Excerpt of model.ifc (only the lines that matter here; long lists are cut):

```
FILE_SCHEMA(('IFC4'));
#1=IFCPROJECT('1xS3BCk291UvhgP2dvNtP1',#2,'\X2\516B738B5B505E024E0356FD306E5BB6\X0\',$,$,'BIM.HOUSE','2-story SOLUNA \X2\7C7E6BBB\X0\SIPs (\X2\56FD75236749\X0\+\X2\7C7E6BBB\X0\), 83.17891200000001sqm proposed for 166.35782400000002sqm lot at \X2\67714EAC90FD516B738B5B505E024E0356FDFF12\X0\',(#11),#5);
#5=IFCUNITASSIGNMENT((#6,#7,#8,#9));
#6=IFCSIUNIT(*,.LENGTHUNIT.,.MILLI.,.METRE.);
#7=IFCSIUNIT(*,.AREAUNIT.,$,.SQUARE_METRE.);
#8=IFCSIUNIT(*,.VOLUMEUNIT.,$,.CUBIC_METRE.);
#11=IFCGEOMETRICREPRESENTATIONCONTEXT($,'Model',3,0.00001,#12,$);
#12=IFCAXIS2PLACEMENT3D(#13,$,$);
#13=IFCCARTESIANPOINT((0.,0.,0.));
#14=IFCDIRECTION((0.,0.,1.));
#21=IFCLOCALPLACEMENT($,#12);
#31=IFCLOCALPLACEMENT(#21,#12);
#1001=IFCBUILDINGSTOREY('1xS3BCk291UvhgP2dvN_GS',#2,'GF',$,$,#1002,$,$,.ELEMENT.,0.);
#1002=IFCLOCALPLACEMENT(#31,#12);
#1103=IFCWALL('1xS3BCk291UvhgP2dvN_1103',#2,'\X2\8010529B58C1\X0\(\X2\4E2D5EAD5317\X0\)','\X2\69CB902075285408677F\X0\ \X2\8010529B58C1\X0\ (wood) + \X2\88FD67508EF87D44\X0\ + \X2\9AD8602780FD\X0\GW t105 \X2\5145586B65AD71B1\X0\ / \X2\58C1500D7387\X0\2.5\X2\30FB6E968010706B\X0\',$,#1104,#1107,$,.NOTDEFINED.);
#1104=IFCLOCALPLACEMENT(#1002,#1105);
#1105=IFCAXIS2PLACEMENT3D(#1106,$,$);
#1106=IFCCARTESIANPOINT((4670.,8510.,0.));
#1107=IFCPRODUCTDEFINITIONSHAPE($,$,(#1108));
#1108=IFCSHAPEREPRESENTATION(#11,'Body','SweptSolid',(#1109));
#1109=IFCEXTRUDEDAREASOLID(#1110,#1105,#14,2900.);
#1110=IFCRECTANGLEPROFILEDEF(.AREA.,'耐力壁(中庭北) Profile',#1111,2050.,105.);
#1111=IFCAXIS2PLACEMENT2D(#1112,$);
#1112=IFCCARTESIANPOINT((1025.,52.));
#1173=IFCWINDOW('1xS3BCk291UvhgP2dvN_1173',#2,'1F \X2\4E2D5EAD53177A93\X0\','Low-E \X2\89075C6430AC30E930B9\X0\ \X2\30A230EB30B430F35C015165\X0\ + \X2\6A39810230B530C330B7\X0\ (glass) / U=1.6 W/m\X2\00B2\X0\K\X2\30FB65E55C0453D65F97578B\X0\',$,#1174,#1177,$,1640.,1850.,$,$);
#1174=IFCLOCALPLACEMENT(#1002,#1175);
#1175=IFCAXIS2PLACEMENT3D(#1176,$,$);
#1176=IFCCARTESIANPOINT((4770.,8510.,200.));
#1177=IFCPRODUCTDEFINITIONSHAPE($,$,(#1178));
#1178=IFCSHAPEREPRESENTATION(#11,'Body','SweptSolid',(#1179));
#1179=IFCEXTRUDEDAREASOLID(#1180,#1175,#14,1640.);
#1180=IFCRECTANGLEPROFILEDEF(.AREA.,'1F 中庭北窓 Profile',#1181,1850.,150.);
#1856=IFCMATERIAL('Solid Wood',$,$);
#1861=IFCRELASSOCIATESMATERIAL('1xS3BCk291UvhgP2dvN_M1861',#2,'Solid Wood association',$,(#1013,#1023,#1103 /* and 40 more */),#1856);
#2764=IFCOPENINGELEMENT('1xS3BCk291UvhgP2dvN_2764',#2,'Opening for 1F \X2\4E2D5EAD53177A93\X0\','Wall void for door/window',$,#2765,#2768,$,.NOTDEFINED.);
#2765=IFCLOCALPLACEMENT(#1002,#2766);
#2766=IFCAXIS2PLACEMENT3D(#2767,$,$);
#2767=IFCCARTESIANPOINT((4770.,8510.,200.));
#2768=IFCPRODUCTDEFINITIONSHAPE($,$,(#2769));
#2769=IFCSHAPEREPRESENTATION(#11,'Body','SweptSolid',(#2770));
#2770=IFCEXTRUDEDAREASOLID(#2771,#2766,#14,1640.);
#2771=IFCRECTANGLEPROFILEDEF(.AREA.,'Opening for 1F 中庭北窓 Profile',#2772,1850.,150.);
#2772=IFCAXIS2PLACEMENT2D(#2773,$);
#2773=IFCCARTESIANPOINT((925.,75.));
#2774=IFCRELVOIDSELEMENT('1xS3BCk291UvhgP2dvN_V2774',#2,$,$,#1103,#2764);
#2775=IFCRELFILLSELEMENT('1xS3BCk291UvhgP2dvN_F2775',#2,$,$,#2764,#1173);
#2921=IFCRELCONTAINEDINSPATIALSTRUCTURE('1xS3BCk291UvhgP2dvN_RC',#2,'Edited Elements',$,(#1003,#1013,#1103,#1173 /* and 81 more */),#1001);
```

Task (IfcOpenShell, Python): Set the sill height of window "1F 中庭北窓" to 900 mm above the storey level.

```python
import numpy as np
import ifcopenshell
import ifcopenshell.api.geometry
import ifcopenshell.geom
import ifcopenshell.util.element
import ifcopenshell.util.placement
import ifcopenshell.util.shape
import ifcopenshell.util.unit

model = ifcopenshell.open("model.ifc")
unit_scale = ifcopenshell.util.unit.calculate_unit_scale(model)

window = model.by_guid("1xS3BCk291UvhgP2dvN_1173")
opening = window.FillsVoids[0].RelatingOpeningElement
storey = ifcopenshell.util.element.get_container(window, ifc_class="IfcBuildingStorey")
level = ifcopenshell.util.placement.get_local_placement(storey.ObjectPlacement)[2, 3]

# The opening's origin need not be at the sill, so measure its lowest point.
shape = ifcopenshell.geom.create_shape(ifcopenshell.geom.settings(), opening)
bottom = ifcopenshell.util.shape.get_shape_bottom_elevation(shape, shape.geometry) / unit_scale
dz = level + 0.9 / unit_scale - bottom

shift = np.array([0.0, 0.0, dz])
# The window is not placed relative to its opening, so move both.
for product in (opening, window):
    matrix = ifcopenshell.util.placement.get_local_placement(product.ObjectPlacement)
    matrix[:3, 3] += shift
    ifcopenshell.api.geometry.edit_object_placement(model, product=product, matrix=matrix, is_si=False)

print(f"moved by {dz * unit_scale:+.3f} m")

model.write("model_edited.ifc")
```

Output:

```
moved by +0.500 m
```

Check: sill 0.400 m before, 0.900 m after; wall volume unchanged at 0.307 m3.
